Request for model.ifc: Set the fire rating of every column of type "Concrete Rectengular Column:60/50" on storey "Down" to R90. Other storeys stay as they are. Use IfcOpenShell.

First a look at what the model holds.

```python
import ifcopenshell
import ifcopenshell.util.element

model = ifcopenshell.open("model.ifc")
print(model.schema)
storey = next(s for s in model.by_type("IfcBuildingStorey") if s.Name == "Down")
columns = [e for e in ifcopenshell.util.element.get_decomposition(storey) if e.is_a("IfcColumn")]
seen = {}
for e in columns:
    element_type = ifcopenshell.util.element.get_type(e)
    key = (element_type.Name if element_type != e and element_type else None, ifcopenshell.util.element.get_pset(e, "Pset_ColumnCommon", "FireRating"))
    seen[key] = seen.get(key, 0) + 1
for (name, value), count in sorted(seen.items(), key=str):
    print(count, "x", name, "|", value)
```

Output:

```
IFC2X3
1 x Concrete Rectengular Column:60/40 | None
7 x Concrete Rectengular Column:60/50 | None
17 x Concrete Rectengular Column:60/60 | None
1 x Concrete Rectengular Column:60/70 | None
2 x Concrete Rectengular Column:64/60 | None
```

```python
import ifcopenshell
import ifcopenshell.api.pset
import ifcopenshell.util.element

model = ifcopenshell.open("model.ifc")

storey = next(s for s in model.by_type("IfcBuildingStorey") if s.Name == "Down")
columns = [e for e in ifcopenshell.util.element.get_decomposition(storey) if e.is_a("IfcColumn")]

count = 0
for e in columns:
    element_type = ifcopenshell.util.element.get_type(e)
    if element_type in (None, e) or element_type.Name != "Concrete Rectengular Column:60/50":
        continue
    # add_pset returns the element's existing set when there is one.
    pset = ifcopenshell.api.pset.add_pset(model, product=e, name="Pset_ColumnCommon")
    ifcopenshell.api.pset.edit_pset(model, pset=pset, properties={"FireRating": "R90"})
    count += 1

print(count, "columns updated")

model.write("model_updated.ifc")
```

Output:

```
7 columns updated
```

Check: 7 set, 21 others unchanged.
